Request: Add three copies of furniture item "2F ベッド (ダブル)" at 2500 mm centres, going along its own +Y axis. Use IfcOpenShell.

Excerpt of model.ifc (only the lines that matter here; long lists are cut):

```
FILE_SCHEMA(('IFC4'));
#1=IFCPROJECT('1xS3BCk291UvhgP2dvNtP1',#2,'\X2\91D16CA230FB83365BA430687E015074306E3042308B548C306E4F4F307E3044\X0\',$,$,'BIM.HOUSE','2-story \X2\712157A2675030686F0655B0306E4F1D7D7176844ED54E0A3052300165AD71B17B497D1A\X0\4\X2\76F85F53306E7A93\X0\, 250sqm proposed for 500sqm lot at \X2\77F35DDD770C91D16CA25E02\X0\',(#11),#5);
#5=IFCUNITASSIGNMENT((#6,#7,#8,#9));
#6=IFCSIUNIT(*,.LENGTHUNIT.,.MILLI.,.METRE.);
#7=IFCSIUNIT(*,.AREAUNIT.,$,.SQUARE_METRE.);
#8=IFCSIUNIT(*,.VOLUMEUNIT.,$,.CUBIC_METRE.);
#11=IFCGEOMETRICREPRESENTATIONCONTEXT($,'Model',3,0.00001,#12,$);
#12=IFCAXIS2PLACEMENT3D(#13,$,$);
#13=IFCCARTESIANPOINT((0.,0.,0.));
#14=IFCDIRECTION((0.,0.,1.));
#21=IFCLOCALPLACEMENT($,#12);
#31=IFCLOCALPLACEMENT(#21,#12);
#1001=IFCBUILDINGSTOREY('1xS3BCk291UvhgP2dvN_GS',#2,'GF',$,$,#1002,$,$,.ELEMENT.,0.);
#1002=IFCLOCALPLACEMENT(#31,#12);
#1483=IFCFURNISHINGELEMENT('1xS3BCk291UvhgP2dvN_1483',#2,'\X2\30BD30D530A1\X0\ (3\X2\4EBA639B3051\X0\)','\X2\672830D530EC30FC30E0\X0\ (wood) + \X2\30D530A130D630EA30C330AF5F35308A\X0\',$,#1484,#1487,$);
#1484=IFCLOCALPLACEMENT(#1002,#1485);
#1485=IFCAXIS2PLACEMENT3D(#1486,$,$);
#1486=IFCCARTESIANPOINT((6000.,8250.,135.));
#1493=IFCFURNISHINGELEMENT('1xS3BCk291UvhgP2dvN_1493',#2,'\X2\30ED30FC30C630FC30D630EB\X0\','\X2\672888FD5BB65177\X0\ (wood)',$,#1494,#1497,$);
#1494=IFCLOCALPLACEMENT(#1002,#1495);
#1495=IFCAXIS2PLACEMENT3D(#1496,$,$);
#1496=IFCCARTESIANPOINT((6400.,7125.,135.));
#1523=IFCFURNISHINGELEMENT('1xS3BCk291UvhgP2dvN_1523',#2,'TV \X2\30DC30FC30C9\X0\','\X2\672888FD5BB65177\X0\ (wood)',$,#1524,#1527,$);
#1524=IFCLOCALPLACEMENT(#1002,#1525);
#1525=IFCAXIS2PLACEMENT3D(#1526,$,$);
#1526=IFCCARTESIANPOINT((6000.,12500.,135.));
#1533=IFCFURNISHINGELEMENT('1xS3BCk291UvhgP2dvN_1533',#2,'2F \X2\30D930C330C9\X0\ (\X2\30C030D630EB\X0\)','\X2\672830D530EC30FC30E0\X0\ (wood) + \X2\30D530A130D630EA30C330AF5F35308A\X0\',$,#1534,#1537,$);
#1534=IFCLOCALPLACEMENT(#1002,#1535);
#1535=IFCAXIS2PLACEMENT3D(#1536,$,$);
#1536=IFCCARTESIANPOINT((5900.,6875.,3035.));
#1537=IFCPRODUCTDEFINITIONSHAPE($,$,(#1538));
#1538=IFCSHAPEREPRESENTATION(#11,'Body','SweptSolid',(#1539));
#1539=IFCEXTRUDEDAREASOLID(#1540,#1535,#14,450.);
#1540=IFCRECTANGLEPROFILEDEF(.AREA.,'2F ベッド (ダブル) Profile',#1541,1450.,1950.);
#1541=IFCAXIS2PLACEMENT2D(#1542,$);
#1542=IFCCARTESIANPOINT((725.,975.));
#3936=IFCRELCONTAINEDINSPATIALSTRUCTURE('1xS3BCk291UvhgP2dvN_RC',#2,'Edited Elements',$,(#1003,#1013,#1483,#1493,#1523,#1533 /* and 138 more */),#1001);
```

```python
import ifcopenshell
import ifcopenshell.api.geometry
import ifcopenshell.api.root
import ifcopenshell.util.element
import ifcopenshell.util.placement
import ifcopenshell.util.unit

model = ifcopenshell.open("model.ifc")
unit_scale = ifcopenshell.util.unit.calculate_unit_scale(model)


def reuse_history(source, copy):
    """copy_class also copies each property set's owner history, people and application; keep the originals."""
    for rel in copy.IsDefinedBy:
        if rel.is_a("IfcRelDefinesByProperties") and (history := rel.RelatingPropertyDefinition.OwnerHistory):
            rel.RelatingPropertyDefinition.OwnerHistory = source.OwnerHistory
            ifcopenshell.util.element.remove_deep2(model, history)


source = model.by_guid("1xS3BCk291UvhgP2dvN_1533")
base = ifcopenshell.util.placement.get_local_placement(source.ObjectPlacement)
step = base[:3, 1] * 2.5 / unit_scale

for i in range(1, 4):
    copy = ifcopenshell.api.root.copy_class(model, product=source)
    copy.Representation = ifcopenshell.util.element.copy_deep(
        model, source.Representation, exclude=["IfcGeometricRepresentationContext", "IfcRepresentationMap"]
    )
    reuse_history(source, copy)
    matrix = base.copy()
    matrix[:3, 3] += i * step
    print("added at", matrix[:3, 3].round(3) + 0.0)
    ifcopenshell.api.geometry.edit_object_placement(model, product=copy, matrix=matrix, is_si=False)

model.write("model_v2.ifc")
```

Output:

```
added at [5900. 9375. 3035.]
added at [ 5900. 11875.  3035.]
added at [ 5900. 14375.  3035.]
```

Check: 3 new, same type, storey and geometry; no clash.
